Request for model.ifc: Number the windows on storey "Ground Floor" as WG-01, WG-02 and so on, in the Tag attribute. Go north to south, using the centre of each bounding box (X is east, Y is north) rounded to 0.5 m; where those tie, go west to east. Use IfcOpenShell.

First a look at what the model holds.

```python
import ifcopenshell
import ifcopenshell.util.element
import ifcopenshell.util.placement

model = ifcopenshell.open("model.ifc")
print(model.schema)
storey = next(s for s in model.by_type("IfcBuildingStorey") if s.Name == "Ground Floor")
windows = [e for e in ifcopenshell.util.element.get_decomposition(storey) if e.is_a("IfcWindow")]
for e in sorted(windows, key=lambda e: e.id()):
    origin = ifcopenshell.util.placement.get_local_placement(e.ObjectPlacement)[:3, 3]
    print(e.id(), e.Tag, e.Name, origin.round(2) + 0.0, sep=" | ")
```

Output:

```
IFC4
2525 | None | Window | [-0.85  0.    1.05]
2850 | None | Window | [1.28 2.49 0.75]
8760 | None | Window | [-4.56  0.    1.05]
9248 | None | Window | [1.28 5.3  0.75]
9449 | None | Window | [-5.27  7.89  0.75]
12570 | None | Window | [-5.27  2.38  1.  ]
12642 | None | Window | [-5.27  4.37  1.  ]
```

```python
import ifcopenshell
import ifcopenshell.geom
import ifcopenshell.util.element
import ifcopenshell.util.shape

model = ifcopenshell.open("model.ifc")
settings = ifcopenshell.geom.settings()
settings.set("use-world-coords", True)


def centre(element):
    shape = ifcopenshell.geom.create_shape(settings, element)
    return ifcopenshell.util.shape.get_bbox_centroid(shape.geometry)


storey = next(s for s in model.by_type("IfcBuildingStorey") if s.Name == "Ground Floor")
windows = [e for e in ifcopenshell.util.element.get_decomposition(storey) if e.is_a("IfcWindow")]

# Insertion points can sit at a corner or the storey origin, so sort by the geometry (in metres).
centres = {e: centre(e) for e in windows}
windows.sort(key=lambda e: (-round(centres[e][1] / 0.5), centres[e][0]))

for i, e in enumerate(windows, start=1):
    number = f"WG-{i:02d}"
    e.Tag = number
    print(e.id(), number)

model.write("model_updated.ifc")
```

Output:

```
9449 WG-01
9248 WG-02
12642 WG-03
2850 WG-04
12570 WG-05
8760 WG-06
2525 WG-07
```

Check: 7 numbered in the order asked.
